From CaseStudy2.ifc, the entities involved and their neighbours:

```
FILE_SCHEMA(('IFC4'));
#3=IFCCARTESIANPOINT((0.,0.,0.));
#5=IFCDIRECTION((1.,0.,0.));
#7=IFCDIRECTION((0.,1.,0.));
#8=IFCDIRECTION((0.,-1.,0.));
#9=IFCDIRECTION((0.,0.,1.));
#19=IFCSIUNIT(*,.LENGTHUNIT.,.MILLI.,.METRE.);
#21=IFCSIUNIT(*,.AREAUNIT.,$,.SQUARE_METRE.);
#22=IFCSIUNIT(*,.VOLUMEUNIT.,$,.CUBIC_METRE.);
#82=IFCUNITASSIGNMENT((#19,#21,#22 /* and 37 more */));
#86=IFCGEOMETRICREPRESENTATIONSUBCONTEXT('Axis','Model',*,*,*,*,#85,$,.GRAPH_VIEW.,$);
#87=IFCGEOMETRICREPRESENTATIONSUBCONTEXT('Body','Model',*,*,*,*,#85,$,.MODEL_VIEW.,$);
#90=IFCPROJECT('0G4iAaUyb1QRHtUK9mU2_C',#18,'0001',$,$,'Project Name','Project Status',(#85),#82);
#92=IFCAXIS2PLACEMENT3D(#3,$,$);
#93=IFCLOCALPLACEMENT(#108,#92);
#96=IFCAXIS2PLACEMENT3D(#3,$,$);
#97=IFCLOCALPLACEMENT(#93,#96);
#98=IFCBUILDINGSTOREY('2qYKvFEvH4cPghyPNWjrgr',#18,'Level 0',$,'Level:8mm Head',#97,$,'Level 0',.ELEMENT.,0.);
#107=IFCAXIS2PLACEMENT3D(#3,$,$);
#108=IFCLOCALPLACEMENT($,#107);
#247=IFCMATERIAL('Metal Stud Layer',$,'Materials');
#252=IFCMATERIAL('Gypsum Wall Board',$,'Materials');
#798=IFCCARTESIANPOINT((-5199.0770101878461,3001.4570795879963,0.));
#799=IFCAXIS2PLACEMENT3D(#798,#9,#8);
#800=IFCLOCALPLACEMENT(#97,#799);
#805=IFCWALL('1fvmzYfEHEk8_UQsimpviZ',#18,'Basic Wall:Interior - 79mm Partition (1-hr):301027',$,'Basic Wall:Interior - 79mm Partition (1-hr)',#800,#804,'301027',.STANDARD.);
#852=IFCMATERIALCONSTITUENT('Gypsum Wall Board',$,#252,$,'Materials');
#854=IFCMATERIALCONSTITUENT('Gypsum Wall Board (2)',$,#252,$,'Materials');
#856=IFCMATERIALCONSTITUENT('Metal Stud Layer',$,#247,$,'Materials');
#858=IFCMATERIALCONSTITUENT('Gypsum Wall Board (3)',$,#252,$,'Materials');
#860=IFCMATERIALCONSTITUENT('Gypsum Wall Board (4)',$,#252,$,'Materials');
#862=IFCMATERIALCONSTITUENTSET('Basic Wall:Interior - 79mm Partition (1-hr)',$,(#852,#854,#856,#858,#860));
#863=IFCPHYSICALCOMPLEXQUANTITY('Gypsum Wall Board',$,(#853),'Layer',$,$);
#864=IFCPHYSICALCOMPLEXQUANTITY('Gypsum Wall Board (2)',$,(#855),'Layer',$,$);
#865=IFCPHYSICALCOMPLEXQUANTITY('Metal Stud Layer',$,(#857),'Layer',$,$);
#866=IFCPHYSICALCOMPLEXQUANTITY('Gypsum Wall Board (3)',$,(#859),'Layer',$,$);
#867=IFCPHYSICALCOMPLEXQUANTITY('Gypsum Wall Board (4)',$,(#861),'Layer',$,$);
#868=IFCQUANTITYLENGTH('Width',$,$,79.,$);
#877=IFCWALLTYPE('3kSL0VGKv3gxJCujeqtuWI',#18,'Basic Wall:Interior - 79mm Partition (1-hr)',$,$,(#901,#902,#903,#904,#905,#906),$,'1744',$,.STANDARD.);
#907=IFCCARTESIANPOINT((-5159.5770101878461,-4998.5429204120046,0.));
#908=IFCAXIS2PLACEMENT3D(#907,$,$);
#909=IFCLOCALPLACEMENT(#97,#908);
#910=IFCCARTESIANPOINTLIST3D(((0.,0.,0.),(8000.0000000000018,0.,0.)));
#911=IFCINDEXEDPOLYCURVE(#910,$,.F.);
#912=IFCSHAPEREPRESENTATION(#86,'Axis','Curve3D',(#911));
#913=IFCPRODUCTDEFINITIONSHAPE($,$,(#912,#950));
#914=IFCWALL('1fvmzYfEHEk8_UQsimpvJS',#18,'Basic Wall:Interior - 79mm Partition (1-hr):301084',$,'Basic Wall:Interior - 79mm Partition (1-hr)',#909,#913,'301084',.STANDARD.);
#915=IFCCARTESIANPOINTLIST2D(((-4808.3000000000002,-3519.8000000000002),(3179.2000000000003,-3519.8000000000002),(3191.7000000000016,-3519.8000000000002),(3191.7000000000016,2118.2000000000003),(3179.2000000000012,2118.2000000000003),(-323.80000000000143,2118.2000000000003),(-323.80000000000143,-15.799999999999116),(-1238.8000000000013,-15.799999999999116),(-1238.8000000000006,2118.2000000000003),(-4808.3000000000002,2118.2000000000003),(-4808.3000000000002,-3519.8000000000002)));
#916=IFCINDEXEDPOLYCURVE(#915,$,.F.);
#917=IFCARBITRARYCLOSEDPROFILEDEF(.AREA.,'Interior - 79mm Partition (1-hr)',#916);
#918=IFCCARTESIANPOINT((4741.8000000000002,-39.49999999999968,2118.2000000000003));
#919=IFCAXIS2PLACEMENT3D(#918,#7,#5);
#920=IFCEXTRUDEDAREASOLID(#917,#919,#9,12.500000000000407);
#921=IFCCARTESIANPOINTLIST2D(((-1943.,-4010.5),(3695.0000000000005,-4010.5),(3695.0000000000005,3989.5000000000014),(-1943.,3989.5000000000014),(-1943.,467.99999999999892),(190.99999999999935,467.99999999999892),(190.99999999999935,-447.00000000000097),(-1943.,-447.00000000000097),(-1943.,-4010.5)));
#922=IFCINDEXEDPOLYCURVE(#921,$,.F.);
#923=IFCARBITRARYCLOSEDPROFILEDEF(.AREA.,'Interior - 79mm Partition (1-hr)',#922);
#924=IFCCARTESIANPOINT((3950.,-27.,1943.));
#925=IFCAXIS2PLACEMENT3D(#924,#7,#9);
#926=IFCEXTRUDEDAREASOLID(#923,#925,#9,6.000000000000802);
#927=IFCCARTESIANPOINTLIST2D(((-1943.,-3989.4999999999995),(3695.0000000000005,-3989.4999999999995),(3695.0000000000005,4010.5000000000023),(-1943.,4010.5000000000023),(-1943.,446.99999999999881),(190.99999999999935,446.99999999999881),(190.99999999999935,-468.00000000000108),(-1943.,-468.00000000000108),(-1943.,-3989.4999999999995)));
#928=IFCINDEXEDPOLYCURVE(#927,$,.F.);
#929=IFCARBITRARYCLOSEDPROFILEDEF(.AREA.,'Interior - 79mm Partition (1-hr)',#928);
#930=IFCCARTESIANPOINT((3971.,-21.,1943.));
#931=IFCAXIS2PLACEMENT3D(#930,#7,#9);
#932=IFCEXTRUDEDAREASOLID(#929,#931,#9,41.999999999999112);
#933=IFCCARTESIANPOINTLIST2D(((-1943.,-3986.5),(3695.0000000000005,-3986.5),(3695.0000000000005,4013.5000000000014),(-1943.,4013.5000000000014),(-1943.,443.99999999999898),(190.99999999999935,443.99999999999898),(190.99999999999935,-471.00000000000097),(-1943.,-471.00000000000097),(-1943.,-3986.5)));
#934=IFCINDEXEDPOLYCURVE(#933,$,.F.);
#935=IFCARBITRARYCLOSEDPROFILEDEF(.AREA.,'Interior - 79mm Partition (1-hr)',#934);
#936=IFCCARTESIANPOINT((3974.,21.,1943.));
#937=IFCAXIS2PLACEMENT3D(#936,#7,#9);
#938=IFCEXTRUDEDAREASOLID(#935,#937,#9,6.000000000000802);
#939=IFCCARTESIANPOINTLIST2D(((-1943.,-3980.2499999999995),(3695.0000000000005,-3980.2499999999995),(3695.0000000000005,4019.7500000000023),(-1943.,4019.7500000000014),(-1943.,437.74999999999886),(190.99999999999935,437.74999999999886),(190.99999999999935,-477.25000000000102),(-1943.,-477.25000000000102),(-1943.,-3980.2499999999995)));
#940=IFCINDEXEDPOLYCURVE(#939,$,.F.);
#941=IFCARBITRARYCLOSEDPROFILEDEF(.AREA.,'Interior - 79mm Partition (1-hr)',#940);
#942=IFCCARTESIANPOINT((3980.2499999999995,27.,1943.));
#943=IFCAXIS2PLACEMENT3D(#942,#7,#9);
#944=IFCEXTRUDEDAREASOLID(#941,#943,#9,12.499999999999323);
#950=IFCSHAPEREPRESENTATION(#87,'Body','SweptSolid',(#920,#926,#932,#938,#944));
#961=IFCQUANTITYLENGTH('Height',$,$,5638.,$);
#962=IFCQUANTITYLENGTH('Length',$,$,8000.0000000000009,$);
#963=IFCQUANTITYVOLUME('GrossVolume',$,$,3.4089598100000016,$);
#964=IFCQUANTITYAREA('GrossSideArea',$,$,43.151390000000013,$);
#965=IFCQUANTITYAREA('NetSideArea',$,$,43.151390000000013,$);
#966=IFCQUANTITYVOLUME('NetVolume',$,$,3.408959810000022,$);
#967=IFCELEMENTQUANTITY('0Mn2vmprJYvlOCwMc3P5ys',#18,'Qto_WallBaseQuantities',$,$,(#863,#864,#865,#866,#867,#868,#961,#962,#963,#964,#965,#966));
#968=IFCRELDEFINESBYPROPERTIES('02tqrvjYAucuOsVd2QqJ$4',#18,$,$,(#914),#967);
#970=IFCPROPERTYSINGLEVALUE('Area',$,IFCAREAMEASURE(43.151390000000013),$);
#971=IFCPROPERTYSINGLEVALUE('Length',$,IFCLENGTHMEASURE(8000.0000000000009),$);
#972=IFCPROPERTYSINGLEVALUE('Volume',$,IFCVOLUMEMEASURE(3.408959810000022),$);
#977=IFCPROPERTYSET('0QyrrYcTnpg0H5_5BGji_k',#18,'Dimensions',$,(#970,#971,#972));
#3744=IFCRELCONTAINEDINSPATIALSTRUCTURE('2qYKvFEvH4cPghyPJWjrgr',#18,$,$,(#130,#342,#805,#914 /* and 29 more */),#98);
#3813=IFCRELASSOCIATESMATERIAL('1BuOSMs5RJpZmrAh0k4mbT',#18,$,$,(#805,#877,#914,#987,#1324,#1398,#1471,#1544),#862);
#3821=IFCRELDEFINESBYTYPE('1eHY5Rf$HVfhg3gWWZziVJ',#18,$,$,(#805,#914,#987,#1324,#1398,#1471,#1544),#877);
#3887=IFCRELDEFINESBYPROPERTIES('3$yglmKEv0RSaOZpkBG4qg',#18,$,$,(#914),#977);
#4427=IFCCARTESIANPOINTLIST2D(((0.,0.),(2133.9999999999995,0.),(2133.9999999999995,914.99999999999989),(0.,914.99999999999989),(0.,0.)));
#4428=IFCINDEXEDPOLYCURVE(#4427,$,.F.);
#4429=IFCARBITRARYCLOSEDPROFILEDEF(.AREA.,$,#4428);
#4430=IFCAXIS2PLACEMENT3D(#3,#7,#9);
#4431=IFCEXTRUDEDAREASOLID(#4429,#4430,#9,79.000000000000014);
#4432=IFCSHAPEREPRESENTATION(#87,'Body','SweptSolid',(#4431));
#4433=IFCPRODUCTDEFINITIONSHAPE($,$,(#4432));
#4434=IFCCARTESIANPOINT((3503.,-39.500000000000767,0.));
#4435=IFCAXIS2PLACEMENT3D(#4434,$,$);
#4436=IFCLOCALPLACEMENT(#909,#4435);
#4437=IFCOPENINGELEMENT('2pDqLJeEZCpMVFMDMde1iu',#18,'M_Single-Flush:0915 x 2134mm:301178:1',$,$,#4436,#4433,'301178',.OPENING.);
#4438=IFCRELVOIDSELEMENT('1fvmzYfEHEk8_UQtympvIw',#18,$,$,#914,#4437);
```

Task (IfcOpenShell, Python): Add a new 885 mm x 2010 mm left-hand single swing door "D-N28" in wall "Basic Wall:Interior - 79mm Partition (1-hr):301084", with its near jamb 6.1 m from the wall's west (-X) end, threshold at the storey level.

```python
import numpy as np
import ifcopenshell
import ifcopenshell.api.feature
import ifcopenshell.api.geometry
import ifcopenshell.api.pset
import ifcopenshell.api.root
import ifcopenshell.api.spatial
import ifcopenshell.geom
import ifcopenshell.util.element
import ifcopenshell.util.placement
import ifcopenshell.util.representation
import ifcopenshell.util.shape
import ifcopenshell.util.unit

model = ifcopenshell.open("CaseStudy2.ifc")
unit_scale = ifcopenshell.util.unit.calculate_unit_scale(model)
area_scale = ifcopenshell.util.unit.calculate_unit_scale(model, "AREAUNIT")
volume_scale = ifcopenshell.util.unit.calculate_unit_scale(model, "VOLUMEUNIT")
settings = ifcopenshell.geom.settings()


def volume(element):
    """Net volume in cubic metres, openings subtracted."""
    shape = ifcopenshell.geom.create_shape(settings, element)
    return ifcopenshell.util.shape.get_volume(shape.geometry)


wall = model.by_id(914)
storey = ifcopenshell.util.element.get_container(wall, ifc_class="IfcBuildingStorey")
context = ifcopenshell.util.representation.get_context(model, "Model", "Body", "MODEL_VIEW")
before = volume(wall)

width, height, from_end, sill = 0.885, 2.01, 6.1, 0.0  # metres

# The wall runs along its own X axis, and the end named is its -X end.
wall_shape = ifcopenshell.geom.create_shape(settings, wall)
x, y, z = ifcopenshell.util.shape.get_vertices(wall_shape.geometry).T
start = x.min() + from_end
face, thickness = float(y.min()), float(y.max() - y.min())
wall_matrix = ifcopenshell.util.placement.get_local_placement(wall.ObjectPlacement)
level = ifcopenshell.util.placement.get_local_placement(storey.ObjectPlacement)[2, 3]


def in_wall(x, y):
    """Placement at x, y metres in the wall's axes, at sill height."""
    matrix = wall_matrix.copy()
    matrix[:, 3] = wall_matrix @ np.array([x / unit_scale, y / unit_scale, 0.0, 1.0])
    matrix[2, 3] = level + sill / unit_scale
    return matrix


# Opening: a box that overshoots both wall faces by 50 mm.
opening = ifcopenshell.api.root.create_entity(model, ifc_class="IfcOpeningElement", predefined_type="OPENING")
box = ifcopenshell.api.geometry.add_wall_representation(
    model, context=context, length=width, height=height, thickness=thickness + 0.1
)
ifcopenshell.api.geometry.assign_representation(model, product=opening, representation=box)
ifcopenshell.api.geometry.edit_object_placement(model, product=opening, matrix=in_wall(start, face - 0.05), is_si=False)
ifcopenshell.api.feature.add_feature(model, feature=opening, element=wall)

door = ifcopenshell.api.root.create_entity(model, ifc_class="IfcDoor", name="D-N28", predefined_type="DOOR")
door.OverallWidth, door.OverallHeight = width / unit_scale, height / unit_scale
door.OperationType = "SINGLE_SWING_LEFT"
body = ifcopenshell.api.geometry.add_door_representation(
    model,
    context=context,
    overall_width=door.OverallWidth,
    overall_height=door.OverallHeight,
    operation_type="SINGLE_SWING_LEFT",
    lining_properties={"LiningDepth": thickness / unit_scale, "ThresholdDepth": thickness / unit_scale},
)
ifcopenshell.api.geometry.assign_representation(model, product=door, representation=body)
ifcopenshell.api.spatial.assign_container(model, products=[door], relating_structure=storey)
ifcopenshell.api.feature.add_filling(model, opening=opening, element=door)

# The lining spans the wall, so the door starts at the wall face.
ifcopenshell.api.geometry.edit_object_placement(model, product=door, matrix=in_wall(start, face), is_si=False)

after = volume(wall)

# Update the wall's stored quantities.
qto = model.by_id(ifcopenshell.util.element.get_pset(wall, "Qto_WallBaseQuantities", should_inherit=False)["id"])
ifcopenshell.api.pset.edit_qto(model, qto=qto, properties={
    "NetSideArea": after / thickness / area_scale,
    "NetVolume": after / volume_scale,
})
pset = model.by_id(ifcopenshell.util.element.get_pset(wall, "Dimensions", should_inherit=False)["id"])
ifcopenshell.api.pset.edit_pset(model, pset=pset, properties={
    "Area": model.create_entity("IfcAreaMeasure", after / thickness / area_scale),
    "Volume": model.create_entity("IfcVolumeMeasure", after / volume_scale),
})

print(f"wall volume {before:.3f} -> {after:.3f} m3")

model.write("CaseStudy2_rev.ifc")
```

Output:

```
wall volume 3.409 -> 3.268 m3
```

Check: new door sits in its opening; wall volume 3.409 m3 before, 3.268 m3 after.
